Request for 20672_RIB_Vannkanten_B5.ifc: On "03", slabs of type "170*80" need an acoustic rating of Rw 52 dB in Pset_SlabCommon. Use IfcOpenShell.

First a look at what the model holds.

```python
import ifcopenshell
import ifcopenshell.util.element

model = ifcopenshell.open("20672_RIB_Vannkanten_B5.ifc")
print(model.schema)
storey = next(s for s in model.by_type("IfcBuildingStorey") if s.Name == "03")
slabs = [e for e in ifcopenshell.util.element.get_decomposition(storey) if e.is_a("IfcSlab")]
seen = {}
for e in slabs:
    element_type = ifcopenshell.util.element.get_type(e)
    key = (element_type.Name if element_type != e and element_type else None, ifcopenshell.util.element.get_pset(e, "Pset_SlabCommon", "AcousticRating"))
    seen[key] = seen.get(key, 0) + 1
for (name, value), count in sorted(seen.items(), key=str):
    print(count, "x", name, "|", value)
```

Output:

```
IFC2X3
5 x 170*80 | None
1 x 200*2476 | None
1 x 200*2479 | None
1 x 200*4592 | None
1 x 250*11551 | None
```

```python
import ifcopenshell
import ifcopenshell.api.pset
import ifcopenshell.util.element

model = ifcopenshell.open("20672_RIB_Vannkanten_B5.ifc")

storey = next(s for s in model.by_type("IfcBuildingStorey") if s.Name == "03")
slabs = [e for e in ifcopenshell.util.element.get_decomposition(storey) if e.is_a("IfcSlab")]

count = 0
for e in slabs:
    element_type = ifcopenshell.util.element.get_type(e)
    if element_type in (None, e) or element_type.Name != "170*80":
        continue
    # add_pset returns the element's existing set when there is one.
    pset = ifcopenshell.api.pset.add_pset(model, product=e, name="Pset_SlabCommon")
    ifcopenshell.api.pset.edit_pset(model, pset=pset, properties={"AcousticRating": "Rw 52 dB"})
    count += 1

print(count, "slabs updated")

model.write("20672_RIB_Vannkanten_B5_edited.ifc")
```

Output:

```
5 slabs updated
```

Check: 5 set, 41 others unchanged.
